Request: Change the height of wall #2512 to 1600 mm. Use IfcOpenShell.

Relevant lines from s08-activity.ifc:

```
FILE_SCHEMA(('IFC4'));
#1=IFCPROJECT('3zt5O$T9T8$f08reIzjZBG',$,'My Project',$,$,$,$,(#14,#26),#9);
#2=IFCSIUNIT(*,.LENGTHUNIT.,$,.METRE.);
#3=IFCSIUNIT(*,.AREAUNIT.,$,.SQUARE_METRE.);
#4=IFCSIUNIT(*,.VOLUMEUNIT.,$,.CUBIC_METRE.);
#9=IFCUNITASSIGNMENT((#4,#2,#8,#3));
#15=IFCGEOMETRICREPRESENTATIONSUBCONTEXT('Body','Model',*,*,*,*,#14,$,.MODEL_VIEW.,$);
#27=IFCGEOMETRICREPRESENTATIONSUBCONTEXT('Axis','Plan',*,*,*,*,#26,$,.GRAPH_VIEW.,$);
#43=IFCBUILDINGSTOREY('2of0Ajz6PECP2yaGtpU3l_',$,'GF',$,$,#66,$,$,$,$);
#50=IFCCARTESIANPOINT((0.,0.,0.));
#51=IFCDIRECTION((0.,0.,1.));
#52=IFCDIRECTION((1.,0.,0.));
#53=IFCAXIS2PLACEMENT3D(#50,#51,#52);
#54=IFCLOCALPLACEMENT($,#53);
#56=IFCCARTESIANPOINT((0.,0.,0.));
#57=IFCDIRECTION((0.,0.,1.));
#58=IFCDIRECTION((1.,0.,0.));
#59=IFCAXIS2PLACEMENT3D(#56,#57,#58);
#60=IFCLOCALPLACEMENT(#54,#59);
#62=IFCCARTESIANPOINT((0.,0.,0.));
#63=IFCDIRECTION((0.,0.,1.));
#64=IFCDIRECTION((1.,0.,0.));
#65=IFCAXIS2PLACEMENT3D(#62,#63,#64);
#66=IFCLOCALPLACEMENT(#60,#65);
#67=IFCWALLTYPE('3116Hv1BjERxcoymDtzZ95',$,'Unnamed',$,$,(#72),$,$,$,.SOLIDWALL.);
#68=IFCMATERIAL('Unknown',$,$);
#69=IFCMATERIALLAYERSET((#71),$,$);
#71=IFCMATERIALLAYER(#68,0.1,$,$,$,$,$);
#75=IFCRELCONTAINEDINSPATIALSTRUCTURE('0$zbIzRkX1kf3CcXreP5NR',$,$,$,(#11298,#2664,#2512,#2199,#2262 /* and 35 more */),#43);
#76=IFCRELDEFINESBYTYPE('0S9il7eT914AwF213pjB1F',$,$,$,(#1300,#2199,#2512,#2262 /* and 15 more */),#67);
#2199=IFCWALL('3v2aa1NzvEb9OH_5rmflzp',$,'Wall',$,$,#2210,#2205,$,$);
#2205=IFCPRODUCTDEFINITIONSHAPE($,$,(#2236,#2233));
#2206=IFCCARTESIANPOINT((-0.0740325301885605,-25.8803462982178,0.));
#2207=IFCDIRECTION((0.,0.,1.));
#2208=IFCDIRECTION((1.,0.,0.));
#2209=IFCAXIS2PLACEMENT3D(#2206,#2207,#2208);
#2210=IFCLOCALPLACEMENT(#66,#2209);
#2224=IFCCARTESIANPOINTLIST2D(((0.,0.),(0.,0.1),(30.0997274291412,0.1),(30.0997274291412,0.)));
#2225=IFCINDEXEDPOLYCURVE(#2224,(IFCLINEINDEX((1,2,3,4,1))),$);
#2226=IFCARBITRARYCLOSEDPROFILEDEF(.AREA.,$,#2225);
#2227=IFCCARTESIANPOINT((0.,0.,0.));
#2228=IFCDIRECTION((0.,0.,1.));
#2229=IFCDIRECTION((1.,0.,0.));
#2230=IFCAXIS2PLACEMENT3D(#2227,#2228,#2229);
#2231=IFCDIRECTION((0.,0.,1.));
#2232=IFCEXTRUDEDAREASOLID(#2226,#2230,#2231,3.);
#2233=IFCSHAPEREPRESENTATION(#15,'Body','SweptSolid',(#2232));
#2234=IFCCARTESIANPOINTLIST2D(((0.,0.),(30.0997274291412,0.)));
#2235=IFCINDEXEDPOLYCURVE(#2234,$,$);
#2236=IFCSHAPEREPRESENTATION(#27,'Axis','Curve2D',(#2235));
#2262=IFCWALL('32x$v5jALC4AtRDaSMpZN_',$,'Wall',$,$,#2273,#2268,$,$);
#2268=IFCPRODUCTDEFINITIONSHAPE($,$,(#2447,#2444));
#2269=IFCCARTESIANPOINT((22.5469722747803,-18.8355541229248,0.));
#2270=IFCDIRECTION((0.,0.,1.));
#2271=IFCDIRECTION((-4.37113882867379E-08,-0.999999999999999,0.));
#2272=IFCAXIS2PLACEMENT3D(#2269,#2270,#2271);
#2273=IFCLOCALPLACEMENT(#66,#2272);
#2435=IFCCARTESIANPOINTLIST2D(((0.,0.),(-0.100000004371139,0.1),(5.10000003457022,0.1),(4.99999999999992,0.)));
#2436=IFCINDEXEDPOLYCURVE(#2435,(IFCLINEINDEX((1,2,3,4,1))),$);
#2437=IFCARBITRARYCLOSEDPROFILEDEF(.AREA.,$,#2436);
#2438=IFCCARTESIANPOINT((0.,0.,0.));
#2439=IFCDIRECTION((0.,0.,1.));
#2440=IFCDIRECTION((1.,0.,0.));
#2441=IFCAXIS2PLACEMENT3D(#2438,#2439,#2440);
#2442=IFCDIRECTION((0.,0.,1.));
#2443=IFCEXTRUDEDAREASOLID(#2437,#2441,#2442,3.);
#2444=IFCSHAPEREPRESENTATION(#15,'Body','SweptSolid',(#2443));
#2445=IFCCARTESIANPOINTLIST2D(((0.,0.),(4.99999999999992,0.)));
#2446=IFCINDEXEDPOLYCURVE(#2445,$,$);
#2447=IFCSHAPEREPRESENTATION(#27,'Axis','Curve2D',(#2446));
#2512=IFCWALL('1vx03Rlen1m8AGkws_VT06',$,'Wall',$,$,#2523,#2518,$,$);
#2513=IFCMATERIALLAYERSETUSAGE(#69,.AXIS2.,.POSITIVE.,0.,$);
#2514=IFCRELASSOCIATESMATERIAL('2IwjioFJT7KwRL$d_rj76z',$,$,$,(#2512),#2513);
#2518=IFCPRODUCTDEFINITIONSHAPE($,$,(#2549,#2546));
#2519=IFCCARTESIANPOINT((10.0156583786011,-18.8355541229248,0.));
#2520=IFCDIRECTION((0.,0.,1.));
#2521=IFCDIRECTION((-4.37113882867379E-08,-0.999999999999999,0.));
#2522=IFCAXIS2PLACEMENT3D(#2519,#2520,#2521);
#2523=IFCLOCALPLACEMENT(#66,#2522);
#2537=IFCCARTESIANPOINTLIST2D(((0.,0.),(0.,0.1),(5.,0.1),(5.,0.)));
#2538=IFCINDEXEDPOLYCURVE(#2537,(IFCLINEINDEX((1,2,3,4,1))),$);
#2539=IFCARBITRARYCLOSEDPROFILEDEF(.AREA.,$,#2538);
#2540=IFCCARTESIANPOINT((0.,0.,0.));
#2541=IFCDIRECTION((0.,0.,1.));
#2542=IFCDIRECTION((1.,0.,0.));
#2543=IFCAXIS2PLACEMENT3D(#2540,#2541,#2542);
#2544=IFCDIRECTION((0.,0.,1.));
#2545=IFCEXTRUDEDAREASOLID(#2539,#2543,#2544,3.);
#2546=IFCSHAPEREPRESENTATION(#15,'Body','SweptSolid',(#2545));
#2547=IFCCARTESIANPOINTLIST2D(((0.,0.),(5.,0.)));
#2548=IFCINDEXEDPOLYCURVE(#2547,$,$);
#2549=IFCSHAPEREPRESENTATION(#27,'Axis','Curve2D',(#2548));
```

```python
import ifcopenshell
import ifcopenshell.geom
import ifcopenshell.util.representation
import ifcopenshell.util.shape
import ifcopenshell.util.unit

model = ifcopenshell.open("s08-activity.ifc")
unit_scale = ifcopenshell.util.unit.calculate_unit_scale(model)
settings = ifcopenshell.geom.settings()


def volume(element):
    """Net volume in cubic metres, openings subtracted."""
    shape = ifcopenshell.geom.create_shape(settings, element)
    return ifcopenshell.util.shape.get_volume(shape.geometry)


wall = model.by_id(2512)
before = volume(wall)

body = ifcopenshell.util.representation.get_representation(wall, "Model", "Body")
solid = body.Items[0]
old_height = solid.Depth
solid.Depth = 1.6 / unit_scale
after = volume(wall)

print(f"height {old_height:g} -> {solid.Depth:g}, volume {before:.3f} -> {after:.3f} m3")

model.write("s08-activity-out.ifc")
```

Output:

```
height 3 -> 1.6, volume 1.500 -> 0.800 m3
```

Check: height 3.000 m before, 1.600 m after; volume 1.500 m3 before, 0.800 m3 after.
